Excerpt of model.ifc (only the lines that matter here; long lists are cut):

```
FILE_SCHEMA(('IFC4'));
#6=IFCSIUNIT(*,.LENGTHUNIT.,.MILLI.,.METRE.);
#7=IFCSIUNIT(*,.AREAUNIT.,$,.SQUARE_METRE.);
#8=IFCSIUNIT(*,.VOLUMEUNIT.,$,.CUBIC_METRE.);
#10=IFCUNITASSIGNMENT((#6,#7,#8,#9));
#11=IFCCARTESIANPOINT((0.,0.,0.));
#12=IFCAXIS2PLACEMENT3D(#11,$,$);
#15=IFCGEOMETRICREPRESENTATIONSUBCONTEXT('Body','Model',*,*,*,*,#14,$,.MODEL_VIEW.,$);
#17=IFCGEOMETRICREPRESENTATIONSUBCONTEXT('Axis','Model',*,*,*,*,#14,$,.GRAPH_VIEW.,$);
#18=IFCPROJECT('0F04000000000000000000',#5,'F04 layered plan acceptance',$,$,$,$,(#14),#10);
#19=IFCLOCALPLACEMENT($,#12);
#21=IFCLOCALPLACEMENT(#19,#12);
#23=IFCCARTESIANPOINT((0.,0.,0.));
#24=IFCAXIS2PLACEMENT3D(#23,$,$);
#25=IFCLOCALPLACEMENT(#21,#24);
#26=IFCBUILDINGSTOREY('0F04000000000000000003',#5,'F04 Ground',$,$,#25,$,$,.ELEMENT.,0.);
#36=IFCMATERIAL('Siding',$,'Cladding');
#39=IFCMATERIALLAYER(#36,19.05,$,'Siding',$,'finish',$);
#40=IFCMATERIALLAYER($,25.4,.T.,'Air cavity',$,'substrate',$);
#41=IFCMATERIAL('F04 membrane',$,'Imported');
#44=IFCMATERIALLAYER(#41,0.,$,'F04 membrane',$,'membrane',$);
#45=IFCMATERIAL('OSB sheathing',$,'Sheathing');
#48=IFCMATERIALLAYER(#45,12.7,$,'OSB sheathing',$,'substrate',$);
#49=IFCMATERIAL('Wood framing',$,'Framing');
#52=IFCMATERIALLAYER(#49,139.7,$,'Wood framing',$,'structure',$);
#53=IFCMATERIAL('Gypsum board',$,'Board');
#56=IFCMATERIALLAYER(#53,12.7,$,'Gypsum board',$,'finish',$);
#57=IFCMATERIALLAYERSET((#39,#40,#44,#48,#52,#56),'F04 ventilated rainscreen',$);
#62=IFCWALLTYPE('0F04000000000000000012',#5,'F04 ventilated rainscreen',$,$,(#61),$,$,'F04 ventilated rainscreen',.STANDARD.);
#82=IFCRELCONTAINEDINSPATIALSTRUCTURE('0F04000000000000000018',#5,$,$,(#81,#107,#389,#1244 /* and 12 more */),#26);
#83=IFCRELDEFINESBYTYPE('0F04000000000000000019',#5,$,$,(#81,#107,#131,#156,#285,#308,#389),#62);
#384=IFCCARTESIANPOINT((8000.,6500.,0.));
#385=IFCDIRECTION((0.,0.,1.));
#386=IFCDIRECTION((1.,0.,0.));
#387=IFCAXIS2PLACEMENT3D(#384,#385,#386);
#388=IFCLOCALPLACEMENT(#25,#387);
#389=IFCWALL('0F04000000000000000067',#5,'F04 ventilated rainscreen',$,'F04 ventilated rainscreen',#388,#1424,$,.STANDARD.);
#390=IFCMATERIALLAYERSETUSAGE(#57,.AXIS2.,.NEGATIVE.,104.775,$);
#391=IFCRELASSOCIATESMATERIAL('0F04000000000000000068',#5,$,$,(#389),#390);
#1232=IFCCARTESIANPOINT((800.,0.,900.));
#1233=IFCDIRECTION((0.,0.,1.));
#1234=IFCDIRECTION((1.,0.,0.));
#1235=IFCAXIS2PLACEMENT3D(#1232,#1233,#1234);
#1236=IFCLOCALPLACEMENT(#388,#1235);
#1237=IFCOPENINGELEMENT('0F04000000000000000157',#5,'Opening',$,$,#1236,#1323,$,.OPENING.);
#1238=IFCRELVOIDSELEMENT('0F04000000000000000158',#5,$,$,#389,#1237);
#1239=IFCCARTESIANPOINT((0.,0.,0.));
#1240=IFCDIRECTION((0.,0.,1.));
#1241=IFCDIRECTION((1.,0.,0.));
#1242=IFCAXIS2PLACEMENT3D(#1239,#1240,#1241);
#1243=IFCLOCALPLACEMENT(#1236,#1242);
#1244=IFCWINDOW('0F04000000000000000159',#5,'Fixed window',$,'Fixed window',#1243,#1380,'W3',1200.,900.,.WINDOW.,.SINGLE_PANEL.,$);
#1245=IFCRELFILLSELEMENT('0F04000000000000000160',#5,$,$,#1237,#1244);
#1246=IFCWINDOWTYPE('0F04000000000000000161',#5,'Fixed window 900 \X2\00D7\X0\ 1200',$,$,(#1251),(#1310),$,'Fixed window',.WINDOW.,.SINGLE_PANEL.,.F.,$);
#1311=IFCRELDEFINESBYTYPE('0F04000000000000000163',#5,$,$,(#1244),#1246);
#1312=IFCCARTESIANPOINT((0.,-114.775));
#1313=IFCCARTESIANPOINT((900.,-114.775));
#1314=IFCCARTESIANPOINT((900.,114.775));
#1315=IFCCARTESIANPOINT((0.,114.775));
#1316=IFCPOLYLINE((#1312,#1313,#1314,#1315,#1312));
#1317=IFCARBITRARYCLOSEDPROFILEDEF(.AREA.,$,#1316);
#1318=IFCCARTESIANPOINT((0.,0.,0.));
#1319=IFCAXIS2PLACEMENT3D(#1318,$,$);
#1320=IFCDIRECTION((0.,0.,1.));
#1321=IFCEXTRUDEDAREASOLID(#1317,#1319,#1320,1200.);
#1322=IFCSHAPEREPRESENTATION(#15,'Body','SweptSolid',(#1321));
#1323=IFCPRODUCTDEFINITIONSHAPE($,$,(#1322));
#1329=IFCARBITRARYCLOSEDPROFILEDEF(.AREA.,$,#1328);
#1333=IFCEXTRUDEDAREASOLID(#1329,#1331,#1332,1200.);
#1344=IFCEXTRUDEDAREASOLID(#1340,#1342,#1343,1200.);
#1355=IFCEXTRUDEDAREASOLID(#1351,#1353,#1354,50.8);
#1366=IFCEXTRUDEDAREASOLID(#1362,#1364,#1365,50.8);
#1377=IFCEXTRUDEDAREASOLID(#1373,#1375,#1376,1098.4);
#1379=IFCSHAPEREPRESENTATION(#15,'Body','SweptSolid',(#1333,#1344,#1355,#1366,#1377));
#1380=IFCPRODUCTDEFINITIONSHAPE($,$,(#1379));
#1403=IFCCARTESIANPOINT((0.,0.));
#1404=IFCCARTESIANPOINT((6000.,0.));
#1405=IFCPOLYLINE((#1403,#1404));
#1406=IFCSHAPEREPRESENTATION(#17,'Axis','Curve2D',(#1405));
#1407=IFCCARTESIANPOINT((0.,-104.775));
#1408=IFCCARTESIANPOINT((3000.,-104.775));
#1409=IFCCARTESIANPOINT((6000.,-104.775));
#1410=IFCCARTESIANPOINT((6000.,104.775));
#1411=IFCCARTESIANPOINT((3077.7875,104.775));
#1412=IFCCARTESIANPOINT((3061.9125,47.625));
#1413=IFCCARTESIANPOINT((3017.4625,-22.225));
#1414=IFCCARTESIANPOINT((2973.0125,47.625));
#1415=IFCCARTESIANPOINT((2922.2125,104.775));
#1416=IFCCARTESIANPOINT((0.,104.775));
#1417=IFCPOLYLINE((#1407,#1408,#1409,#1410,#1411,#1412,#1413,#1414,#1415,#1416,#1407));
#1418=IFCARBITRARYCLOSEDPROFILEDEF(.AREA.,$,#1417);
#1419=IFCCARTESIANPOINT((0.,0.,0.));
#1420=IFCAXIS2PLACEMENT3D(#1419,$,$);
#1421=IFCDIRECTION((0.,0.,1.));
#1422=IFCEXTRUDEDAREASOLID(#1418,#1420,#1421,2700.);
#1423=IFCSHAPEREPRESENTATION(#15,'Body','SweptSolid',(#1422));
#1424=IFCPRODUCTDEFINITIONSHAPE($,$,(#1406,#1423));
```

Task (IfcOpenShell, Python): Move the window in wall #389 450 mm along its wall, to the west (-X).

```python
import ifcopenshell
import ifcopenshell.api.geometry
import ifcopenshell.util.placement
import ifcopenshell.util.unit

model = ifcopenshell.open("model.ifc")
unit_scale = ifcopenshell.util.unit.calculate_unit_scale(model)

window = model.by_guid("0F04000000000000000159")
opening = window.FillsVoids[0].RelatingOpeningElement
wall = opening.VoidsElements[0].RelatingBuildingElement

wall_matrix = ifcopenshell.util.placement.get_local_placement(wall.ObjectPlacement)
shift = wall_matrix[:3, 0] * -0.45 / unit_scale
before = ifcopenshell.util.placement.get_local_placement(window.ObjectPlacement)[:3, 3].copy()

# The window is placed relative to its opening, so it follows when the opening moves.
matrix = ifcopenshell.util.placement.get_local_placement(opening.ObjectPlacement)
matrix[:3, 3] += shift
ifcopenshell.api.geometry.edit_object_placement(
    model, product=opening, matrix=matrix, is_si=False, should_transform_children=True
)

after = ifcopenshell.util.placement.get_local_placement(window.ObjectPlacement)[:3, 3]
print("window moved by", (after - before).round(3) + 0.0)

model.write("model_edited.ifc")
```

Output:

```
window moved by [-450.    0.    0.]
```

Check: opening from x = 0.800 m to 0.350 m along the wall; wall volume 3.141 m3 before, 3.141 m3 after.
